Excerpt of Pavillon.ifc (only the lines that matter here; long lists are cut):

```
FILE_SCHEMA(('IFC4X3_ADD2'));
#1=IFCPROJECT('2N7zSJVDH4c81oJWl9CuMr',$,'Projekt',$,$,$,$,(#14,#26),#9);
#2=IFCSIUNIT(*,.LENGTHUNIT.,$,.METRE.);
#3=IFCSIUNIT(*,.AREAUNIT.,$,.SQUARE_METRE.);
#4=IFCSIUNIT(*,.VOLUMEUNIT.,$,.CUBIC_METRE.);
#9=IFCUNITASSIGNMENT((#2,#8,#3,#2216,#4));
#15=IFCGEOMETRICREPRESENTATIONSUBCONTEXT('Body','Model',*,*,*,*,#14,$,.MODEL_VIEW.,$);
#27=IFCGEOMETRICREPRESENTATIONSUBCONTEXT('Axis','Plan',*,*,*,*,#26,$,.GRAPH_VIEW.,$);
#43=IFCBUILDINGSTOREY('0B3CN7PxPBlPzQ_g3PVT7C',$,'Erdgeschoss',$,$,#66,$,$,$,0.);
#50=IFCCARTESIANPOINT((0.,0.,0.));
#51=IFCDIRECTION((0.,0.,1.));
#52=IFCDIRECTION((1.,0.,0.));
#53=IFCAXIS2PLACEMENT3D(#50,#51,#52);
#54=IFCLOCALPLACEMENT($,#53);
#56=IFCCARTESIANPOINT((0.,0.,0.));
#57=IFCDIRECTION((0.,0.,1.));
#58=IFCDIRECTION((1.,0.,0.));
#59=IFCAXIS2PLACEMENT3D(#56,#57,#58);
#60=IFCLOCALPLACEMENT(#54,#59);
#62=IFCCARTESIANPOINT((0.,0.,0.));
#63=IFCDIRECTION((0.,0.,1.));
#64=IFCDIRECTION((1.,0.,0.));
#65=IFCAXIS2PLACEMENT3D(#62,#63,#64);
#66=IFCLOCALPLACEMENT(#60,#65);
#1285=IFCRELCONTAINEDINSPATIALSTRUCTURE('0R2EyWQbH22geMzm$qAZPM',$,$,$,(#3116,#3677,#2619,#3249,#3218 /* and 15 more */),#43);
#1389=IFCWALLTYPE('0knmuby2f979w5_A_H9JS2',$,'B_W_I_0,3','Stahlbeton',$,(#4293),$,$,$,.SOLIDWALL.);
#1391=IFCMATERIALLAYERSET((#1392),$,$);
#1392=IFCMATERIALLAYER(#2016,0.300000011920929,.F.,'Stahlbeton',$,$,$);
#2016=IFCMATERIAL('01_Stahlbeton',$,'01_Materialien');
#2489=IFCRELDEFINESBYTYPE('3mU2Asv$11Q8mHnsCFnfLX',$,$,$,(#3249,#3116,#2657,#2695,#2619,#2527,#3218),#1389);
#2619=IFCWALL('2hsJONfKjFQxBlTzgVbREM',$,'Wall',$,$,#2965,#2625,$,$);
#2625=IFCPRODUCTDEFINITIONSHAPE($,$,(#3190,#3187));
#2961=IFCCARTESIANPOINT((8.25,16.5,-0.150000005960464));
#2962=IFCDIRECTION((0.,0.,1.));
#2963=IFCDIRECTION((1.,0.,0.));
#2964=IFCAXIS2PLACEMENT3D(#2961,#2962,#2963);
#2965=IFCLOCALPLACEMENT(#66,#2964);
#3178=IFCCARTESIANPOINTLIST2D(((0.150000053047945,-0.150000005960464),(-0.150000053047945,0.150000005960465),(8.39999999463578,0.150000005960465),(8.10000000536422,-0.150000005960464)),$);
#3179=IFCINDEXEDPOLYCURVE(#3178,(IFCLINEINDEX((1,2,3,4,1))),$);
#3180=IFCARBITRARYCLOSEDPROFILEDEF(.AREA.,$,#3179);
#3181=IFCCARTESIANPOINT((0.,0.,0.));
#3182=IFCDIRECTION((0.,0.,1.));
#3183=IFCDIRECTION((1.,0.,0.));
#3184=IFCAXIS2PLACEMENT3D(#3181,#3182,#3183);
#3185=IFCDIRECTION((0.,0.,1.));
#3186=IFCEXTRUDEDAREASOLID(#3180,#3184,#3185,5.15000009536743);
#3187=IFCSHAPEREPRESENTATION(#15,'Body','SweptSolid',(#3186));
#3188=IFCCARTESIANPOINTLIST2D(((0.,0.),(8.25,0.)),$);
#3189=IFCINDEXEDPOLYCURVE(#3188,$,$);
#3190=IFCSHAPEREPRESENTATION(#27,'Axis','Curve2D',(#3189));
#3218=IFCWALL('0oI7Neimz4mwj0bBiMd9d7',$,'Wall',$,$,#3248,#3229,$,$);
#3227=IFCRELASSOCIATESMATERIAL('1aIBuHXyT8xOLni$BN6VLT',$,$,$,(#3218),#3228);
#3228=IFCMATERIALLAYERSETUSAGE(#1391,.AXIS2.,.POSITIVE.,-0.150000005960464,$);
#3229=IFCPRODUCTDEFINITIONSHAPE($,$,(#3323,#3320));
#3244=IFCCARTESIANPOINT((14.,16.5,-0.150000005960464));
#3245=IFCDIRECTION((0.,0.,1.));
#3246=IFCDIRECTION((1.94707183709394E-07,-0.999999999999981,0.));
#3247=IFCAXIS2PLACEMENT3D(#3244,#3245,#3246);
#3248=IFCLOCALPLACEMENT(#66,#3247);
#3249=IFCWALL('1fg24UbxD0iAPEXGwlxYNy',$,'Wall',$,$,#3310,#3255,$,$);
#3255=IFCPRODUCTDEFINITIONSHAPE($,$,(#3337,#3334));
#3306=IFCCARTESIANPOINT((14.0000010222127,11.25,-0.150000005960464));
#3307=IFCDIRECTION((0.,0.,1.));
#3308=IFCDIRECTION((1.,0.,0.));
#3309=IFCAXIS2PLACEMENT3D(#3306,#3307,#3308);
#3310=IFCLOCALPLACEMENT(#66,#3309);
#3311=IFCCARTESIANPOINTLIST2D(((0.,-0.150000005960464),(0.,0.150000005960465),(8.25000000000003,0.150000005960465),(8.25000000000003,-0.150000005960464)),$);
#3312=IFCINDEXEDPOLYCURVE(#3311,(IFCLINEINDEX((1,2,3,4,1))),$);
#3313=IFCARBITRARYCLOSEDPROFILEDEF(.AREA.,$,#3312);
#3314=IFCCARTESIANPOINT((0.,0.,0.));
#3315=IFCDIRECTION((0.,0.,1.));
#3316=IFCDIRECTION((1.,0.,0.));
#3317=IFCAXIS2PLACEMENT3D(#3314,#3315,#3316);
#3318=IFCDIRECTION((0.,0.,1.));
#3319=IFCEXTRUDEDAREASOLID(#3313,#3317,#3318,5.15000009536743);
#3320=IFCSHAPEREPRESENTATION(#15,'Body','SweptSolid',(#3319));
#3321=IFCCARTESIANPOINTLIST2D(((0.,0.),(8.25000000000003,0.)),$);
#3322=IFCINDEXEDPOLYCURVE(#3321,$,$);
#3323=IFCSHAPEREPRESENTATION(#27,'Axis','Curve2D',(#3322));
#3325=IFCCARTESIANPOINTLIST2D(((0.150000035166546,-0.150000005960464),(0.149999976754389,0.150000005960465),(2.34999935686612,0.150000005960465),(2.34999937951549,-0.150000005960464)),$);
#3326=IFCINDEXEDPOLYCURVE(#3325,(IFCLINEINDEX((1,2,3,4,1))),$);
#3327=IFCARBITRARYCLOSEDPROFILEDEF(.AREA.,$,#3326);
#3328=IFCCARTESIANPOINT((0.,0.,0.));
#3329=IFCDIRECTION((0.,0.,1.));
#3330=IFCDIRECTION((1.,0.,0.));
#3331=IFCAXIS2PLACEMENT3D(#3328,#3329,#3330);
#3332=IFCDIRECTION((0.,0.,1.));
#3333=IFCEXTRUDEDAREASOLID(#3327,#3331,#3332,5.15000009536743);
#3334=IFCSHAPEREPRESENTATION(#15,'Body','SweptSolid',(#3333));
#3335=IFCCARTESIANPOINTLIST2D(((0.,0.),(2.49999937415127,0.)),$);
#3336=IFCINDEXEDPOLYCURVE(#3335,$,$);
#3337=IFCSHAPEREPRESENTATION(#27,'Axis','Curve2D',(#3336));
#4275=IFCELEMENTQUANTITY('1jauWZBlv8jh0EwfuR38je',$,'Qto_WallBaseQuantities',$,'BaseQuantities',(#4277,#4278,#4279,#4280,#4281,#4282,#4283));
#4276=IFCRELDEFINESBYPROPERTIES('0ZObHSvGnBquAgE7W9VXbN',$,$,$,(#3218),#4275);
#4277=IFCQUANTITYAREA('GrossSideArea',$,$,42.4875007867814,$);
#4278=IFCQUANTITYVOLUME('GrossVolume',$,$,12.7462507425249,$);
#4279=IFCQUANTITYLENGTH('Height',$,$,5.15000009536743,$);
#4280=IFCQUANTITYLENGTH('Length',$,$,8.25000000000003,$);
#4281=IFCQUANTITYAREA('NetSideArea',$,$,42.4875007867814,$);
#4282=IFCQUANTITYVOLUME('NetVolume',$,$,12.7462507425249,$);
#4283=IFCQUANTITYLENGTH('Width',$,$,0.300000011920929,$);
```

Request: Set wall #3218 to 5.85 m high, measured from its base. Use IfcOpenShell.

```python
import ifcopenshell
import ifcopenshell.api.pset
import ifcopenshell.geom
import ifcopenshell.util.element
import ifcopenshell.util.representation
import ifcopenshell.util.shape
import ifcopenshell.util.unit

model = ifcopenshell.open("Pavillon.ifc")
unit_scale = ifcopenshell.util.unit.calculate_unit_scale(model)
area_scale = ifcopenshell.util.unit.calculate_unit_scale(model, "AREAUNIT")
volume_scale = ifcopenshell.util.unit.calculate_unit_scale(model, "VOLUMEUNIT")
settings = ifcopenshell.geom.settings()


def volume(element):
    """Net volume in cubic metres, openings subtracted."""
    shape = ifcopenshell.geom.create_shape(settings, element)
    return ifcopenshell.util.shape.get_volume(shape.geometry)


wall = model.by_guid("0oI7Neimz4mwj0bBiMd9d7")
before = volume(wall)

body = ifcopenshell.util.representation.get_representation(wall, "Model", "Body")
solid = body.Items[0]
old_height = solid.Depth
solid.Depth = 5.85
after = volume(wall)
thickness = 0.3  # wall thickness in metres

# Update the stored height, areas and volumes.
qto = model.by_id(ifcopenshell.util.element.get_pset(wall, "Qto_WallBaseQuantities", should_inherit=False)["id"])
ifcopenshell.api.pset.edit_qto(model, qto=qto, properties={
    "GrossSideArea": ifcopenshell.util.element.get_pset(wall, "Qto_WallBaseQuantities", "GrossSideArea") * solid.Depth / old_height,
    "GrossVolume": ifcopenshell.util.element.get_pset(wall, "Qto_WallBaseQuantities", "GrossVolume") * solid.Depth / old_height,
    "Height": solid.Depth,
    "NetSideArea": after / thickness / area_scale,
    "NetVolume": after / volume_scale,
})

print(f"height {old_height:g} -> {solid.Depth:g}, volume {before:.3f} -> {after:.3f} m3")

model.write("Pavillon_rev.ifc")
```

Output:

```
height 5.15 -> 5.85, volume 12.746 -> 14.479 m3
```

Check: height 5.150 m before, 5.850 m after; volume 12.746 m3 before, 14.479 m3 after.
